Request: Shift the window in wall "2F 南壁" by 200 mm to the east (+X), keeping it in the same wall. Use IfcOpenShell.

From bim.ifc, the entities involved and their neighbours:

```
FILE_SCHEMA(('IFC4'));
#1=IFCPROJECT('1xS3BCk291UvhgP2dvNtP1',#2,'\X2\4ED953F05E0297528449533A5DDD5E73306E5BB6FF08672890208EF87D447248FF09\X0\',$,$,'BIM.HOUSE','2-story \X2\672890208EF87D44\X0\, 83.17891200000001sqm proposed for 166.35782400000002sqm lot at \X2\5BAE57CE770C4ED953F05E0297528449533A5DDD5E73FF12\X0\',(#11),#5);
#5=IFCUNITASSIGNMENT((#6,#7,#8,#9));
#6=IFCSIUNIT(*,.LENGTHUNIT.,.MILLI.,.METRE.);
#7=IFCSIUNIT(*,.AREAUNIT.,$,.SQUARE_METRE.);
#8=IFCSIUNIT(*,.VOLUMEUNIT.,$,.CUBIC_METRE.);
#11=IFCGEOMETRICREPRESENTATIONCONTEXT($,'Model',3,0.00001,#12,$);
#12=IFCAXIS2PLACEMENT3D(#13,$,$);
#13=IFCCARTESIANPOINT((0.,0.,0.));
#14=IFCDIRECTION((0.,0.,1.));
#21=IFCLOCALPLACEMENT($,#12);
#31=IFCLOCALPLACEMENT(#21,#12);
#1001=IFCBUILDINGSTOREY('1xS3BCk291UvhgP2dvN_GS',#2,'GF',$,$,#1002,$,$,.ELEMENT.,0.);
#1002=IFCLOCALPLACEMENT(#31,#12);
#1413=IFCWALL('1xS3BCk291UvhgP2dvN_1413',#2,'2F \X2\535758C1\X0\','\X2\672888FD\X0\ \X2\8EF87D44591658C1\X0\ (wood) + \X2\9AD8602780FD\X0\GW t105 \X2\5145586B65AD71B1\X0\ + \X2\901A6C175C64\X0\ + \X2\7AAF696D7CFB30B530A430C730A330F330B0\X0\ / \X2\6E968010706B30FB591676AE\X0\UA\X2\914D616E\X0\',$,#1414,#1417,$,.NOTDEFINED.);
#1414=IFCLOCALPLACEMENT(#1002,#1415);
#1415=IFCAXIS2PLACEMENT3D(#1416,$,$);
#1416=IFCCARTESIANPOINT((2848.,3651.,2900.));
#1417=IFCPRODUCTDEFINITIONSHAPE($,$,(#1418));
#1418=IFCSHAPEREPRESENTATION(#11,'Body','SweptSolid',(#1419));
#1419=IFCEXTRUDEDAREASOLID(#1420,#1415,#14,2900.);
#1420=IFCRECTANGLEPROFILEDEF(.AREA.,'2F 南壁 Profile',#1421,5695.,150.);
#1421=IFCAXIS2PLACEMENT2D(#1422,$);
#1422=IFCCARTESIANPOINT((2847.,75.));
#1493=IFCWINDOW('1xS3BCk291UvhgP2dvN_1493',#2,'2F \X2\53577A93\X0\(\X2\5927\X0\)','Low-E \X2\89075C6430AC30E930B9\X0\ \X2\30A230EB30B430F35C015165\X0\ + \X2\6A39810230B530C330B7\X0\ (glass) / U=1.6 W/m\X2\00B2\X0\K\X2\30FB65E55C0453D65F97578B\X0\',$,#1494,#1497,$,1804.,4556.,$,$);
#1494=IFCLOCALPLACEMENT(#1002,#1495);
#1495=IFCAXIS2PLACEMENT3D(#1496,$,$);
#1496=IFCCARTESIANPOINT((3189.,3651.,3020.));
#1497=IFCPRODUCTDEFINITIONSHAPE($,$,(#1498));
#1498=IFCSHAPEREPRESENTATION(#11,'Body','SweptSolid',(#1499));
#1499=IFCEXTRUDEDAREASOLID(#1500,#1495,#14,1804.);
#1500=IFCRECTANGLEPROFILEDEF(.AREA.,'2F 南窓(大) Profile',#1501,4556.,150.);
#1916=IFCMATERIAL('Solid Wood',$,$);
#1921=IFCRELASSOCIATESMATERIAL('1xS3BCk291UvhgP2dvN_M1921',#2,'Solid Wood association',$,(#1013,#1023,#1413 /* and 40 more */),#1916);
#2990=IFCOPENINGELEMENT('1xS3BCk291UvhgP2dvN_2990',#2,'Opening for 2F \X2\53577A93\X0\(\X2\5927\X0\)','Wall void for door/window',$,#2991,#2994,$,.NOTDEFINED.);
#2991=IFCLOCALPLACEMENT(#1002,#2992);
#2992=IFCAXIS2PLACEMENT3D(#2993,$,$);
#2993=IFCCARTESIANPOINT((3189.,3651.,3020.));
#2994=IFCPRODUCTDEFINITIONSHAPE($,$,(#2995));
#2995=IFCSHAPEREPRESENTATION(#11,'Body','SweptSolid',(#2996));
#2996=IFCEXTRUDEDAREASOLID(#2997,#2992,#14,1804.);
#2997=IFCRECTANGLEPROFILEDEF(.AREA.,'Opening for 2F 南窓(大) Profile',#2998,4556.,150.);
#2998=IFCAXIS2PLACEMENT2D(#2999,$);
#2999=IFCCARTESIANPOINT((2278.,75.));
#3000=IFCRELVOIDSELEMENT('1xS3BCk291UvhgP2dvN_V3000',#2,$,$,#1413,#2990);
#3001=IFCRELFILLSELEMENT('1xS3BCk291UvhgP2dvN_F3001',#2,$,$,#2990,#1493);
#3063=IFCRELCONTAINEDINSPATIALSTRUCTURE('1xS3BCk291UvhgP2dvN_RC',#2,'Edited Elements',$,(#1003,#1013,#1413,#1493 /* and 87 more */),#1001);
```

```python
import ifcopenshell
import ifcopenshell.api.geometry
import ifcopenshell.util.placement
import ifcopenshell.util.unit

model = ifcopenshell.open("bim.ifc")
unit_scale = ifcopenshell.util.unit.calculate_unit_scale(model)

window = model.by_guid("1xS3BCk291UvhgP2dvN_1493")
opening = window.FillsVoids[0].RelatingOpeningElement
wall = opening.VoidsElements[0].RelatingBuildingElement

wall_matrix = ifcopenshell.util.placement.get_local_placement(wall.ObjectPlacement)
shift = wall_matrix[:3, 0] * 0.2 / unit_scale
before = ifcopenshell.util.placement.get_local_placement(window.ObjectPlacement)[:3, 3].copy()

# The window is not placed relative to its opening, so move both.
for product in (opening, window):
    matrix = ifcopenshell.util.placement.get_local_placement(product.ObjectPlacement)
    matrix[:3, 3] += shift
    ifcopenshell.api.geometry.edit_object_placement(model, product=product, matrix=matrix, is_si=False)

after = ifcopenshell.util.placement.get_local_placement(window.ObjectPlacement)[:3, 3]
print("window moved by", (after - before).round(3) + 0.0)

model.write("bim_edited.ifc")
```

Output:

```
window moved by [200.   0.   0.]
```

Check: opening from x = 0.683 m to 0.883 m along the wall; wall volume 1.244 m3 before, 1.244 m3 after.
